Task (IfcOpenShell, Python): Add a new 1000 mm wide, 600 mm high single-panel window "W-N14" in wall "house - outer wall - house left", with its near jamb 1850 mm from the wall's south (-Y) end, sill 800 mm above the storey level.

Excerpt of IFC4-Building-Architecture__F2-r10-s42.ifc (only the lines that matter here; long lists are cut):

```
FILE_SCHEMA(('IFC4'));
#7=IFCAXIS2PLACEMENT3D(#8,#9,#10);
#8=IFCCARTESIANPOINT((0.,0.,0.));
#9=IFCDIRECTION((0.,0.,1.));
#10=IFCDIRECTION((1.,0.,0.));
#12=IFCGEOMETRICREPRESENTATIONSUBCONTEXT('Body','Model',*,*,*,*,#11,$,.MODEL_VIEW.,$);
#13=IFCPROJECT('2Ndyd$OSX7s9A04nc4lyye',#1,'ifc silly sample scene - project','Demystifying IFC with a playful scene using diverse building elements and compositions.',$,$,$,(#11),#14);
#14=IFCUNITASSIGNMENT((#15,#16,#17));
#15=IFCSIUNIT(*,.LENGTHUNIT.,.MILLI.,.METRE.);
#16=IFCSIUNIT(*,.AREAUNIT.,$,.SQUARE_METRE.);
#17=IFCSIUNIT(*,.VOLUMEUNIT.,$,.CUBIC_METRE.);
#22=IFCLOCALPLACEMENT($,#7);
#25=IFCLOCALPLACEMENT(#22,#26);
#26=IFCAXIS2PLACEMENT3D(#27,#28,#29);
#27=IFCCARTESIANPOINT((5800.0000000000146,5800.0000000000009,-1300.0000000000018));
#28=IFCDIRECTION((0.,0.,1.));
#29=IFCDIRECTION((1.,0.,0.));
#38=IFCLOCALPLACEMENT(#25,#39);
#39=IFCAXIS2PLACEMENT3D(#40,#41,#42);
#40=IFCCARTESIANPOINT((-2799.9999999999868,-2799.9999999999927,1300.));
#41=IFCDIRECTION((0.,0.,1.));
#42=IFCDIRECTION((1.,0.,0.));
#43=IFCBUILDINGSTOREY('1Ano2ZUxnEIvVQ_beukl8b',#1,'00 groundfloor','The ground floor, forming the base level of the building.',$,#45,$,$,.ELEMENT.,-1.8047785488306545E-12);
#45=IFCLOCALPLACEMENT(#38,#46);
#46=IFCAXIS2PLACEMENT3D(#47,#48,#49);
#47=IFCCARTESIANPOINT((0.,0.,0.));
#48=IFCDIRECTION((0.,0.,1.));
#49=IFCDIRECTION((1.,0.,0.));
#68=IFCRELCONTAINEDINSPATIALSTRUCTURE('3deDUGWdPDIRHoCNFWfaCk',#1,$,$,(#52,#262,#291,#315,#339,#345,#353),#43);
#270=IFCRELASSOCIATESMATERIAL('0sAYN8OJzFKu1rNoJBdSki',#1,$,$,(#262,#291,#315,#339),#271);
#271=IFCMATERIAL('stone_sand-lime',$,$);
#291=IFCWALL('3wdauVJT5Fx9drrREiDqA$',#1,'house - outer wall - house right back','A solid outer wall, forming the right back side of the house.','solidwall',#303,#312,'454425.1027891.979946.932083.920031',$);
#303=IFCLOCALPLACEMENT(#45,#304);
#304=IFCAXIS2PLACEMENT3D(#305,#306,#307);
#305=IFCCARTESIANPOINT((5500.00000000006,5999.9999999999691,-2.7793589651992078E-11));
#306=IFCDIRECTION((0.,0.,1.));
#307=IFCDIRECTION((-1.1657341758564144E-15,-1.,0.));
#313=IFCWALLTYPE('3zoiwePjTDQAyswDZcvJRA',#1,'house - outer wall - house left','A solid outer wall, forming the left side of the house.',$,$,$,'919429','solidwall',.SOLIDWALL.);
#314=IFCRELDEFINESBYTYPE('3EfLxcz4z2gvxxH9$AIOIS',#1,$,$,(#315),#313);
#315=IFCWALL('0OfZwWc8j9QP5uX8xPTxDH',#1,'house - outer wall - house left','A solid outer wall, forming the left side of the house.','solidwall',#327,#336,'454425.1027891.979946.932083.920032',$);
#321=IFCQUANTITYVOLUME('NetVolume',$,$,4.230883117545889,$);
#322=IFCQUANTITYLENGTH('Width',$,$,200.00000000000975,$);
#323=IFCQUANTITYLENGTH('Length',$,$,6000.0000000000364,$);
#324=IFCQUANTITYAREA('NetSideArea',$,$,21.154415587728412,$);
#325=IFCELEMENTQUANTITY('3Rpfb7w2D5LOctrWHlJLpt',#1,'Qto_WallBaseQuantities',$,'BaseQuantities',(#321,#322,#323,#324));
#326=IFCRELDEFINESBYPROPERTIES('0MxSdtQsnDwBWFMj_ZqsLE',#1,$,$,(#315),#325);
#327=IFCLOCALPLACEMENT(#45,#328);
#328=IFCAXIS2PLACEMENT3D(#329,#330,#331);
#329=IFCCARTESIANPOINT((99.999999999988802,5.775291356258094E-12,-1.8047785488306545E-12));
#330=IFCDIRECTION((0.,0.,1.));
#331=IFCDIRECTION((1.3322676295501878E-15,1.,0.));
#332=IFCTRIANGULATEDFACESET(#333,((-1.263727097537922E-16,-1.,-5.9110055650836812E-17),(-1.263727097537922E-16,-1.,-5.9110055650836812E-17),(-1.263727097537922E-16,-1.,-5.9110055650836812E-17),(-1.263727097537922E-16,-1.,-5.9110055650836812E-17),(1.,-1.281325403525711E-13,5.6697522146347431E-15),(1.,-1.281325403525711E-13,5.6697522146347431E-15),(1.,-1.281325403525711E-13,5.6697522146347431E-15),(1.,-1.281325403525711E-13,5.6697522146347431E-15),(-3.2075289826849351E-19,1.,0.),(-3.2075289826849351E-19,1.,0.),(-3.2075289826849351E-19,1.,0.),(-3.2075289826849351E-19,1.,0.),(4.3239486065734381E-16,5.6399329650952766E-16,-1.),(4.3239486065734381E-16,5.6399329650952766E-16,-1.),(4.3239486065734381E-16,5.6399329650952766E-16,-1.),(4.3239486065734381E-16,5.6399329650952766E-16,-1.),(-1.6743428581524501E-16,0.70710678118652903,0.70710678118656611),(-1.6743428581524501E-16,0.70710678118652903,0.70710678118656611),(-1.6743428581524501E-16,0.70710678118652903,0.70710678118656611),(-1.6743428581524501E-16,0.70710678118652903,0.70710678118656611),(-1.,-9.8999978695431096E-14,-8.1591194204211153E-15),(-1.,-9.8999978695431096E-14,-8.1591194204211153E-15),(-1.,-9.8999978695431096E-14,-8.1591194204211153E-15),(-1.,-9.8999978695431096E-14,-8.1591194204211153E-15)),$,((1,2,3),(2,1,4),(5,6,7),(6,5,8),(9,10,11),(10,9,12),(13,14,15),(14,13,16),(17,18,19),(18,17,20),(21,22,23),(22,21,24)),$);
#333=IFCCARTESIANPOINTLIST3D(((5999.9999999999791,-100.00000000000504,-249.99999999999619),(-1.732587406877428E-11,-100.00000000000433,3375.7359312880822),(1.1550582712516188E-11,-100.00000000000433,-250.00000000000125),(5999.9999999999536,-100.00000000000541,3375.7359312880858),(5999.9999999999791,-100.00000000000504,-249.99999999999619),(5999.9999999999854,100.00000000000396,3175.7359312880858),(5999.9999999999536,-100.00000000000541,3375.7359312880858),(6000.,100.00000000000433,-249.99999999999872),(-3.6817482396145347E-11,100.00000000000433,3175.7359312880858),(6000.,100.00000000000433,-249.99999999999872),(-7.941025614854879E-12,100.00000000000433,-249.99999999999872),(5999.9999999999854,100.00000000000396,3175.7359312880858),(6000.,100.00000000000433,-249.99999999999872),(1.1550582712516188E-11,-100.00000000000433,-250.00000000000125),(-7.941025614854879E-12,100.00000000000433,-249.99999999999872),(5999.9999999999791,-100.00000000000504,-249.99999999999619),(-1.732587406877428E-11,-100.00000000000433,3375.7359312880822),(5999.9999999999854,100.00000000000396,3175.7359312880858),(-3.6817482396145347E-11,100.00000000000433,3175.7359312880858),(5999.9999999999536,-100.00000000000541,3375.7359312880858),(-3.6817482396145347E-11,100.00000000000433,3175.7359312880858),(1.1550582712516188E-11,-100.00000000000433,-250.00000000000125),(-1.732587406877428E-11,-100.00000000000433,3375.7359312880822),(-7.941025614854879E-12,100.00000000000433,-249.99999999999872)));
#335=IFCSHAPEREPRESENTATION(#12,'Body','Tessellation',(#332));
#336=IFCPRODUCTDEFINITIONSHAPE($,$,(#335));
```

```python
import numpy as np
import ifcopenshell
import ifcopenshell.api.feature
import ifcopenshell.api.geometry
import ifcopenshell.api.pset
import ifcopenshell.api.root
import ifcopenshell.api.spatial
import ifcopenshell.geom
import ifcopenshell.util.element
import ifcopenshell.util.placement
import ifcopenshell.util.representation
import ifcopenshell.util.shape
import ifcopenshell.util.unit

model = ifcopenshell.open("IFC4-Building-Architecture__F2-r10-s42.ifc")
unit_scale = ifcopenshell.util.unit.calculate_unit_scale(model)
area_scale = ifcopenshell.util.unit.calculate_unit_scale(model, "AREAUNIT")
volume_scale = ifcopenshell.util.unit.calculate_unit_scale(model, "VOLUMEUNIT")
settings = ifcopenshell.geom.settings()


def volume(element):
    """Net volume in cubic metres, openings subtracted."""
    shape = ifcopenshell.geom.create_shape(settings, element)
    return ifcopenshell.util.shape.get_volume(shape.geometry)


wall = model.by_guid("0OfZwWc8j9QP5uX8xPTxDH")
storey = ifcopenshell.util.element.get_container(wall, ifc_class="IfcBuildingStorey")
context = ifcopenshell.util.representation.get_context(model, "Model", "Body", "MODEL_VIEW")
before = volume(wall)

width, height, from_end, sill = 1, 0.6, 1.85, 0.8  # metres

# The wall runs along its own X axis, and the end named is its -X end.
wall_shape = ifcopenshell.geom.create_shape(settings, wall)
x, y, z = ifcopenshell.util.shape.get_vertices(wall_shape.geometry).T
start = x.min() + from_end
face, thickness = float(y.min()), float(y.max() - y.min())
wall_matrix = ifcopenshell.util.placement.get_local_placement(wall.ObjectPlacement)
level = ifcopenshell.util.placement.get_local_placement(storey.ObjectPlacement)[2, 3]


def in_wall(x, y):
    """Placement at x, y metres in the wall's axes, at sill height."""
    matrix = wall_matrix.copy()
    matrix[:, 3] = wall_matrix @ np.array([x / unit_scale, y / unit_scale, 0.0, 1.0])
    matrix[2, 3] = level + sill / unit_scale
    return matrix


# Opening: a box that overshoots both wall faces by 50 mm.
opening = ifcopenshell.api.root.create_entity(model, ifc_class="IfcOpeningElement", predefined_type="OPENING")
box = ifcopenshell.api.geometry.add_wall_representation(
    model, context=context, length=width, height=height, thickness=thickness + 0.1
)
ifcopenshell.api.geometry.assign_representation(model, product=opening, representation=box)
ifcopenshell.api.geometry.edit_object_placement(model, product=opening, matrix=in_wall(start, face - 0.05), is_si=False)
ifcopenshell.api.feature.add_feature(model, feature=opening, element=wall)

window = ifcopenshell.api.root.create_entity(model, ifc_class="IfcWindow", name="W-N14", predefined_type="WINDOW")
window.OverallWidth, window.OverallHeight = width / unit_scale, height / unit_scale
window.PartitioningType = "SINGLE_PANEL"
body = ifcopenshell.api.geometry.add_window_representation(
    model,
    context=context,
    overall_width=window.OverallWidth,
    overall_height=window.OverallHeight,
    partition_type="SINGLE_PANEL",
)
ifcopenshell.api.geometry.assign_representation(model, product=window, representation=body)
ifcopenshell.api.spatial.assign_container(model, products=[window], relating_structure=storey)
ifcopenshell.api.feature.add_filling(model, opening=opening, element=window)

# Centre the window in the wall's thickness.
ifcopenshell.api.geometry.edit_object_placement(model, product=window, matrix=in_wall(start, face), is_si=False)
window_shape = ifcopenshell.geom.create_shape(settings, window)
depth = ifcopenshell.util.shape.get_vertices(window_shape.geometry)[:, 1]
offset = face + thickness / 2 - (depth.min() + depth.max()) / 2
ifcopenshell.api.geometry.edit_object_placement(model, product=window, matrix=in_wall(start, offset), is_si=False)

after = volume(wall)

# Update the wall's stored quantities.
qto = model.by_id(ifcopenshell.util.element.get_pset(wall, "Qto_WallBaseQuantities", should_inherit=False)["id"])
ifcopenshell.api.pset.edit_qto(model, qto=qto, properties={
    "NetVolume": after / volume_scale,
    "NetSideArea": after / thickness / area_scale,
})

print(f"wall volume {before:.3f} -> {after:.3f} m3")

model.write("IFC4-Building-Architecture__F2-r10-s42_edited.ifc")
```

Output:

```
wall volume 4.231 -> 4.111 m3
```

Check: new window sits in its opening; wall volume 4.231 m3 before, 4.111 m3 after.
